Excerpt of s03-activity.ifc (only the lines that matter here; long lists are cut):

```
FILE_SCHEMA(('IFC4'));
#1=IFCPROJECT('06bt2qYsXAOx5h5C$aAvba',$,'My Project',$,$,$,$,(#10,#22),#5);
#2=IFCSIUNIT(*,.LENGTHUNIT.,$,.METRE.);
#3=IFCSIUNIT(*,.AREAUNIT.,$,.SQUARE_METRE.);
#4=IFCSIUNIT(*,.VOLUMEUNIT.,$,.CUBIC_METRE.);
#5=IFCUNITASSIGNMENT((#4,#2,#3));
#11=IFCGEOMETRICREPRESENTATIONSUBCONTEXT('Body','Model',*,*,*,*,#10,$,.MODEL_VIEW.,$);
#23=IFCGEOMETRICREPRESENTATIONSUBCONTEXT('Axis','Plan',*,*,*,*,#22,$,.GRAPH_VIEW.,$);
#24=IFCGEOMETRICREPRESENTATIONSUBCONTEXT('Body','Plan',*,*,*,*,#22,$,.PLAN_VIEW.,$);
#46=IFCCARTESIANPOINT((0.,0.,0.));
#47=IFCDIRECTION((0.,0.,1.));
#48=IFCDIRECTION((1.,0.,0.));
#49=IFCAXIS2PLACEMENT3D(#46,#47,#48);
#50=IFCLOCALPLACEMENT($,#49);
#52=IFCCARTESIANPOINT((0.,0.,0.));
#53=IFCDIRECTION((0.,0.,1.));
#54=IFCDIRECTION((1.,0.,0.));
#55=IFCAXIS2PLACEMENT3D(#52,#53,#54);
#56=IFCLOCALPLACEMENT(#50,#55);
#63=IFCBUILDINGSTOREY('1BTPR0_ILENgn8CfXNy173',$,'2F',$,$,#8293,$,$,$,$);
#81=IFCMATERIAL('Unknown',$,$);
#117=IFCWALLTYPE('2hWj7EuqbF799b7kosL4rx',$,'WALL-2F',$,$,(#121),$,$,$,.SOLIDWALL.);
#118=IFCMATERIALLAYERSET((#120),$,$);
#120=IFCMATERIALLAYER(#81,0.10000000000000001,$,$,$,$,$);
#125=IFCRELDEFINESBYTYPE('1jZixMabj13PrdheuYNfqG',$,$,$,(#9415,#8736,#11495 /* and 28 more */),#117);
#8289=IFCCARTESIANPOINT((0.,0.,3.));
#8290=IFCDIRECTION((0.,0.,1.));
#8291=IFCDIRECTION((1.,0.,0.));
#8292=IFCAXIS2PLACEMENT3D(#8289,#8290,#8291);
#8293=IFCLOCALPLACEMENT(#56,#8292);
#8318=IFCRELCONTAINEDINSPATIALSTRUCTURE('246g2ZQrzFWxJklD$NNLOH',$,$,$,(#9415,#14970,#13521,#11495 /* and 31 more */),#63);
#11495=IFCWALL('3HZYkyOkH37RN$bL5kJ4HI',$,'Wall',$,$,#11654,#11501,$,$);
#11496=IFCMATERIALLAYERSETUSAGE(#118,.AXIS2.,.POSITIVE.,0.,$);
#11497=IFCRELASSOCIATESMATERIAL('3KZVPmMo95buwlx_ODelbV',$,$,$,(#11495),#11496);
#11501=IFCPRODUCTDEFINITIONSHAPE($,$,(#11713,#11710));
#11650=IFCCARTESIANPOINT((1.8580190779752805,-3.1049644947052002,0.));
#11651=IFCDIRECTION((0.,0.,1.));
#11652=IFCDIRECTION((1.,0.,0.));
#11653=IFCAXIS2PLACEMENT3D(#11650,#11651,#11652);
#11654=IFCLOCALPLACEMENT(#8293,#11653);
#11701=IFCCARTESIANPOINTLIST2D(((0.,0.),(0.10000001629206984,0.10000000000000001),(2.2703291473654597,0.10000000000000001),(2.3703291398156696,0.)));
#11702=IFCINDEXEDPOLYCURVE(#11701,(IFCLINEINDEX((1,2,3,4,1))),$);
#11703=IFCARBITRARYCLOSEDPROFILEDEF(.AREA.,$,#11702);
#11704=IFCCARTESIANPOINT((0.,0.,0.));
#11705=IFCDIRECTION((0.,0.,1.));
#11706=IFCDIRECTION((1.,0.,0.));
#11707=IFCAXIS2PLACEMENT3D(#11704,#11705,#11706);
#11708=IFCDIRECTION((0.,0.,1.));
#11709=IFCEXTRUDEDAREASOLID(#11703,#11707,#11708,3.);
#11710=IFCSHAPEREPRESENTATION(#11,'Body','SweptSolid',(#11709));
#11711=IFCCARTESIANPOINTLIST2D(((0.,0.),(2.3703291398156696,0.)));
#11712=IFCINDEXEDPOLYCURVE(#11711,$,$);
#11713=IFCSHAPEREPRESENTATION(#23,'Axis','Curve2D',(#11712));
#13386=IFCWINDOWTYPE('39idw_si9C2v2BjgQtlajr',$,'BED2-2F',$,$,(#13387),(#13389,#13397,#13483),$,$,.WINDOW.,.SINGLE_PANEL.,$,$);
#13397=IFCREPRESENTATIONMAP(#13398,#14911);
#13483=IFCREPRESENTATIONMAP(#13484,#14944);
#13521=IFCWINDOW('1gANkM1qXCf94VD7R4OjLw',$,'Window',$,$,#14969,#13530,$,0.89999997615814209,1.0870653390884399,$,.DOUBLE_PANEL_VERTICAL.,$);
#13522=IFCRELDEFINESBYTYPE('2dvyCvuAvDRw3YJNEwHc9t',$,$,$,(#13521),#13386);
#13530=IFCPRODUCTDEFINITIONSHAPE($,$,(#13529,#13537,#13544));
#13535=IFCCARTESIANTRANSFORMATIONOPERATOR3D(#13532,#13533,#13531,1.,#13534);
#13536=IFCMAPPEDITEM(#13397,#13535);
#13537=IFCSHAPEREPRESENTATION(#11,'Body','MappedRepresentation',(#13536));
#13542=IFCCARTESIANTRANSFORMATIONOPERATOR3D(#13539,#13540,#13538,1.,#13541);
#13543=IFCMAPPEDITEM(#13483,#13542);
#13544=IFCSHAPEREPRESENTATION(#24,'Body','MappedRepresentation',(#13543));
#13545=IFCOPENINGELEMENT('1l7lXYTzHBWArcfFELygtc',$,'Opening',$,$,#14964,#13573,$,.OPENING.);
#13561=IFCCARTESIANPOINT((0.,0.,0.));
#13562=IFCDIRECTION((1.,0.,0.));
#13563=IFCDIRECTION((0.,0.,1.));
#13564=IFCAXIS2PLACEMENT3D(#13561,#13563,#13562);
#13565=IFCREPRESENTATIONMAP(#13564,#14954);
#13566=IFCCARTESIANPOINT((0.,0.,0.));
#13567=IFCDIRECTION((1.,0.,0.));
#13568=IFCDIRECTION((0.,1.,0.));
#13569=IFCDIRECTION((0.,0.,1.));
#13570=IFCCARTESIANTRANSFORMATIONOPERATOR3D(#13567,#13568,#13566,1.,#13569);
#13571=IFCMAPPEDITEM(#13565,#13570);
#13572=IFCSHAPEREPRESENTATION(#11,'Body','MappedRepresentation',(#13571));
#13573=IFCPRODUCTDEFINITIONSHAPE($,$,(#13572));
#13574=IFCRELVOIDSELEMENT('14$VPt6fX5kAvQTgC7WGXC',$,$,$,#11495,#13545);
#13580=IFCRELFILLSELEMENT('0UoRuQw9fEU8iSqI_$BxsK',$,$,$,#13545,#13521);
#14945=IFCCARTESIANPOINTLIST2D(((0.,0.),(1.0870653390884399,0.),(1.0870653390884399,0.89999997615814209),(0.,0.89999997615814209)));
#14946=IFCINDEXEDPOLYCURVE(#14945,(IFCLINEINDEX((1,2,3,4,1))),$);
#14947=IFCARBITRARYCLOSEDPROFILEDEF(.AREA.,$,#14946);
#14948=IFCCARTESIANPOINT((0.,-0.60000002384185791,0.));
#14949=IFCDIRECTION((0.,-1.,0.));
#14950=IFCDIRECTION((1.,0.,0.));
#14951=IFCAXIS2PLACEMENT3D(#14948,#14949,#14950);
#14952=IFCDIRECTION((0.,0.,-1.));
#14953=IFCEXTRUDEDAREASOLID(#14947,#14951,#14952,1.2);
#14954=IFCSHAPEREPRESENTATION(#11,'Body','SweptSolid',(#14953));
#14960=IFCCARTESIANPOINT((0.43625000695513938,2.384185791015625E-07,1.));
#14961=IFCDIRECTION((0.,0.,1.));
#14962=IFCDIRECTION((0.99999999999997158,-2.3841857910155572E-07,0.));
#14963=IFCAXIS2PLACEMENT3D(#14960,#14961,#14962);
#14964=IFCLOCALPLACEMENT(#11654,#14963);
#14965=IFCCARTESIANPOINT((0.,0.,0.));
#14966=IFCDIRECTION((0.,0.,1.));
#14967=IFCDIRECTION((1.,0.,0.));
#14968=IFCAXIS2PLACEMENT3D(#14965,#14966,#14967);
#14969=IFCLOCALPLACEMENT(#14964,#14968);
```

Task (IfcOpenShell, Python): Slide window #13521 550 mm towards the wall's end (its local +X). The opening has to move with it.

```python
import ifcopenshell
import ifcopenshell.api.geometry
import ifcopenshell.util.placement

model = ifcopenshell.open("s03-activity.ifc")

window = model.by_id(13521)
opening = window.FillsVoids[0].RelatingOpeningElement
wall = opening.VoidsElements[0].RelatingBuildingElement

wall_matrix = ifcopenshell.util.placement.get_local_placement(wall.ObjectPlacement)
shift = wall_matrix[:3, 0] * 0.55
before = ifcopenshell.util.placement.get_local_placement(window.ObjectPlacement)[:3, 3].copy()

# The window is placed relative to its opening, so it follows when the opening moves.
matrix = ifcopenshell.util.placement.get_local_placement(opening.ObjectPlacement)
matrix[:3, 3] += shift
ifcopenshell.api.geometry.edit_object_placement(
    model, product=opening, matrix=matrix, is_si=False, should_transform_children=True
)

after = ifcopenshell.util.placement.get_local_placement(window.ObjectPlacement)[:3, 3]
print("window moved by", (after - before).round(3) + 0.0)

model.write("s03-activity_updated.ifc")
```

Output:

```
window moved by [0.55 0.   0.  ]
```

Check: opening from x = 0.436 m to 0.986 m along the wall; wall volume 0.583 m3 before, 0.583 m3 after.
